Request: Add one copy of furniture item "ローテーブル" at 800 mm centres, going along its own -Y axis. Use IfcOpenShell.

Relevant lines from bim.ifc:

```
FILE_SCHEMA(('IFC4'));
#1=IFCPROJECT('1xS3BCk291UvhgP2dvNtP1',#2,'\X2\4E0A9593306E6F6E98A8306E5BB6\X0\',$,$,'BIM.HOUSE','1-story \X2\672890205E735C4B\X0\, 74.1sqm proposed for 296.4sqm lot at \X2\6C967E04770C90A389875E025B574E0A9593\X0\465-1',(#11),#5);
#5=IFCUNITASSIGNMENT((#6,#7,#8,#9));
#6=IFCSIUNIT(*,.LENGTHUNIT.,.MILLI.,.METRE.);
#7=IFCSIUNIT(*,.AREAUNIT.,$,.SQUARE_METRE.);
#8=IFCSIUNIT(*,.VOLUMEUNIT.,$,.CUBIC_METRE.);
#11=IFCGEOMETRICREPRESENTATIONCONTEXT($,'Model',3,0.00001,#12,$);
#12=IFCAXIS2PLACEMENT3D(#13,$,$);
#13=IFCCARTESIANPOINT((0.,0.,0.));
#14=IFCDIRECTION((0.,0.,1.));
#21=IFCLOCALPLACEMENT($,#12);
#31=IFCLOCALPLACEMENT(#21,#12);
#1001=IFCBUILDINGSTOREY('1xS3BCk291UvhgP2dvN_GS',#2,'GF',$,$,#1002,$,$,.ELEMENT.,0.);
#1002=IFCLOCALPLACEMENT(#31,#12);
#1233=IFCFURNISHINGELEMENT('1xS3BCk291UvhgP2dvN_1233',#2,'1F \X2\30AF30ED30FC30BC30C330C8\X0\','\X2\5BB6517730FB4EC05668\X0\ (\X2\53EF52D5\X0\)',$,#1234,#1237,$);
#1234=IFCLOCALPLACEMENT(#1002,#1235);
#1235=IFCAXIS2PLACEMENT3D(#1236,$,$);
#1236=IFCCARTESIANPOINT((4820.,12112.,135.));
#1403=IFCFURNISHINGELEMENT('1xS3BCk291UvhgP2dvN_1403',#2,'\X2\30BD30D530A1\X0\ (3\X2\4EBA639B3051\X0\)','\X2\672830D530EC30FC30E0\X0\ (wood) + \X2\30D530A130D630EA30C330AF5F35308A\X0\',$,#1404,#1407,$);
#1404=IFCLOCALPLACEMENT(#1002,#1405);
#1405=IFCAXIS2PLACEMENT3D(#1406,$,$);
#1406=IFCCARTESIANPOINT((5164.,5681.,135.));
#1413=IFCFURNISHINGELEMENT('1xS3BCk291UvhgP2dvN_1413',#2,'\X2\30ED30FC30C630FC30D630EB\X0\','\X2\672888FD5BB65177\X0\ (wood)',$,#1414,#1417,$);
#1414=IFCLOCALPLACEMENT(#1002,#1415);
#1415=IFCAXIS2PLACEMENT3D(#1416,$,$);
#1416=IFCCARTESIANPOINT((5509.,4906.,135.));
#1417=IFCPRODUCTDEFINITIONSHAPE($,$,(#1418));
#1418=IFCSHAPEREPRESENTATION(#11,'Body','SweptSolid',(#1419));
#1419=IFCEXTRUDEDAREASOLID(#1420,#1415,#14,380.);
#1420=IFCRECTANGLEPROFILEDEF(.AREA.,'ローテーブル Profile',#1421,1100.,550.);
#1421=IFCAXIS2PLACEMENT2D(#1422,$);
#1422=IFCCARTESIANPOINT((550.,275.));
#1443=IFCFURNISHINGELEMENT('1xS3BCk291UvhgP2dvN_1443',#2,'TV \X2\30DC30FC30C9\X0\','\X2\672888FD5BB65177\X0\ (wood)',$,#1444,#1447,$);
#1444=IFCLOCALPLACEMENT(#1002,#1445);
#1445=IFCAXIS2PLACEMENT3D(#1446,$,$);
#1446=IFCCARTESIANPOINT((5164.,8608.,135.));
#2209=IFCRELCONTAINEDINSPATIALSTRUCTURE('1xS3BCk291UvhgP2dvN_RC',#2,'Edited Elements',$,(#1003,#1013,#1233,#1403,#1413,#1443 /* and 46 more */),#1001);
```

```python
import ifcopenshell
import ifcopenshell.api.geometry
import ifcopenshell.api.root
import ifcopenshell.util.element
import ifcopenshell.util.placement
import ifcopenshell.util.unit

model = ifcopenshell.open("bim.ifc")
unit_scale = ifcopenshell.util.unit.calculate_unit_scale(model)


def reuse_history(source, copy):
    """copy_class also copies each property set's owner history, people and application; keep the originals."""
    for rel in copy.IsDefinedBy:
        if rel.is_a("IfcRelDefinesByProperties") and (history := rel.RelatingPropertyDefinition.OwnerHistory):
            rel.RelatingPropertyDefinition.OwnerHistory = source.OwnerHistory
            ifcopenshell.util.element.remove_deep2(model, history)


source = model.by_guid("1xS3BCk291UvhgP2dvN_1413")
base = ifcopenshell.util.placement.get_local_placement(source.ObjectPlacement)
step = -base[:3, 1] * 0.8 / unit_scale

for i in range(1, 2):
    copy = ifcopenshell.api.root.copy_class(model, product=source)
    copy.Representation = ifcopenshell.util.element.copy_deep(
        model, source.Representation, exclude=["IfcGeometricRepresentationContext", "IfcRepresentationMap"]
    )
    reuse_history(source, copy)
    matrix = base.copy()
    matrix[:3, 3] += i * step
    print("added at", matrix[:3, 3].round(3) + 0.0)
    ifcopenshell.api.geometry.edit_object_placement(model, product=copy, matrix=matrix, is_si=False)

model.write("bim_v2.ifc")
```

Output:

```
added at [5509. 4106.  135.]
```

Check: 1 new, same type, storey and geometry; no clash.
